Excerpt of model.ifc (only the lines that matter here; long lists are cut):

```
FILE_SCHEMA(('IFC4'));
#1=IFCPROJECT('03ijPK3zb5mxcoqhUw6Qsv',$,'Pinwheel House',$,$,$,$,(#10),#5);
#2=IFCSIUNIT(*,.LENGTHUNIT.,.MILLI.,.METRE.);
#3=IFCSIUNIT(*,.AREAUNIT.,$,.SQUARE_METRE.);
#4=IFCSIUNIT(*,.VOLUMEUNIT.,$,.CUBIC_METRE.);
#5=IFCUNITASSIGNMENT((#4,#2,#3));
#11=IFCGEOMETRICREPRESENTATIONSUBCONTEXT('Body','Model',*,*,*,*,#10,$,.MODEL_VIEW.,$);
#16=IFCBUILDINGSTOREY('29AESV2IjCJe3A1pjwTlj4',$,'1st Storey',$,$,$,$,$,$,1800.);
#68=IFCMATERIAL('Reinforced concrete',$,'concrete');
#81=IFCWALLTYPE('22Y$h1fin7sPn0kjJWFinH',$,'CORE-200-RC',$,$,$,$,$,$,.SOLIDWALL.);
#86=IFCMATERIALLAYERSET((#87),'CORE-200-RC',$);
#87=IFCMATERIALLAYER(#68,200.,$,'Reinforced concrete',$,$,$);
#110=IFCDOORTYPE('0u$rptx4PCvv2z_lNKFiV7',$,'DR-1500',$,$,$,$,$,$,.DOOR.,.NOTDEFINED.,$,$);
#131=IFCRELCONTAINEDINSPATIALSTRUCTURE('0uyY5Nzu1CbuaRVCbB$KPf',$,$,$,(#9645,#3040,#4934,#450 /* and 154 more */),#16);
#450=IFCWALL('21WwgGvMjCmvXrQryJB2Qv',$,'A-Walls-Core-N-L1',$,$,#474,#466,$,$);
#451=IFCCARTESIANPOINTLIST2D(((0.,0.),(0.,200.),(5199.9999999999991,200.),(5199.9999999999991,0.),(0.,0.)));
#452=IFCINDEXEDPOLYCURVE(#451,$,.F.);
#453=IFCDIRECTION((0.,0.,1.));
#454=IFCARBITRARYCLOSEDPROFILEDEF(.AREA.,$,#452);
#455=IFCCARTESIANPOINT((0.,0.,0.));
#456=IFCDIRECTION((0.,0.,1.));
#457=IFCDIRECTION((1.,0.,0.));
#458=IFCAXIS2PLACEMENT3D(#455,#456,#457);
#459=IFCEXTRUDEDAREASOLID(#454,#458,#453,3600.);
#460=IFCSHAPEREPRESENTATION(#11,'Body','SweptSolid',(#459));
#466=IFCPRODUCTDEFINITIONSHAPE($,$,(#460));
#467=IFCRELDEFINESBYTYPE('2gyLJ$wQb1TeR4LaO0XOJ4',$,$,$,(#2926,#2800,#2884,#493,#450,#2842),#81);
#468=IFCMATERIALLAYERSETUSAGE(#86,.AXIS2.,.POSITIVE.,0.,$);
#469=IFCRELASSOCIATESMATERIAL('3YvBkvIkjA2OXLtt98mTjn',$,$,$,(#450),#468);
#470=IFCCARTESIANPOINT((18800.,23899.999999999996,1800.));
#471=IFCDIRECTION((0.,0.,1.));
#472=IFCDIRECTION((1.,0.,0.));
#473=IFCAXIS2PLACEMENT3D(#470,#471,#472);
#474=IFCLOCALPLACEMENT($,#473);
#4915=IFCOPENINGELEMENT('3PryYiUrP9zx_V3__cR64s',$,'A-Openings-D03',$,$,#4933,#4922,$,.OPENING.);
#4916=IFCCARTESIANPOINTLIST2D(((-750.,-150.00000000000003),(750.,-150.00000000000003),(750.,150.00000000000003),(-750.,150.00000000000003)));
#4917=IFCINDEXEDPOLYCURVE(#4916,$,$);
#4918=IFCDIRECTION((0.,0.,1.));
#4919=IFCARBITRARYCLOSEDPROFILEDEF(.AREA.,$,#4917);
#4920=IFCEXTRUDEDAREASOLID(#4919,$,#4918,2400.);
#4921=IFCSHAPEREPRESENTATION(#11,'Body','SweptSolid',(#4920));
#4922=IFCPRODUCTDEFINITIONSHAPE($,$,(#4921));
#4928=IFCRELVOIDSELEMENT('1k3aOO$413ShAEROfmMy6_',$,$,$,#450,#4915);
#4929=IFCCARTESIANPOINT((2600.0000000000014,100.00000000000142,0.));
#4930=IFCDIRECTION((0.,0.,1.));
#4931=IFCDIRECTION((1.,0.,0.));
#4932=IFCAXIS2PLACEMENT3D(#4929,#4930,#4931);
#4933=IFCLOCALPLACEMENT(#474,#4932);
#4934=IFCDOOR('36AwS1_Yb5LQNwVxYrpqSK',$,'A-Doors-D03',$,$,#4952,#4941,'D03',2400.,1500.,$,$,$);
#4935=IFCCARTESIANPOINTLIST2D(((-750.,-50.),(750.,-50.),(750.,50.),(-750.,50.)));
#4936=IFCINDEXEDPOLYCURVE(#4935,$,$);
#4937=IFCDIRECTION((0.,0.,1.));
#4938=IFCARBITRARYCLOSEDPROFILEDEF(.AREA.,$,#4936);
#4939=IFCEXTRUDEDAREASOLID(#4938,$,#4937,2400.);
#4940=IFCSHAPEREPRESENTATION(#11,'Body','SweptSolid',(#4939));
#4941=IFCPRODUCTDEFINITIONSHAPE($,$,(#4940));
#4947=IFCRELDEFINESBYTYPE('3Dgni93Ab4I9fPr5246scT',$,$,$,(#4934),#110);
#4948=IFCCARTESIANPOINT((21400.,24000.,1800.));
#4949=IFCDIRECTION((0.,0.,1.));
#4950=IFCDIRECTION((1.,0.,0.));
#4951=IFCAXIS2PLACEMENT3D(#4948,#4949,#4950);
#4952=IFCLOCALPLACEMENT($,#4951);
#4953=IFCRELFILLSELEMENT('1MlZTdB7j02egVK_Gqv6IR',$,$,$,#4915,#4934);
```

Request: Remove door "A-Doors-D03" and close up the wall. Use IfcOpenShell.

```python
import ifcopenshell
import ifcopenshell.api.feature
import ifcopenshell.api.root
import ifcopenshell.geom
import ifcopenshell.util.shape

model = ifcopenshell.open("model.ifc")
settings = ifcopenshell.geom.settings()


def volume(element):
    """Net volume in cubic metres, openings subtracted."""
    shape = ifcopenshell.geom.create_shape(settings, element)
    return ifcopenshell.util.shape.get_volume(shape.geometry)


door = model.by_guid("36AwS1_Yb5LQNwVxYrpqSK")
opening = door.FillsVoids[0].RelatingOpeningElement
wall = opening.VoidsElements[0].RelatingBuildingElement
before = volume(wall)

ifcopenshell.api.root.remove_product(model, product=door)
ifcopenshell.api.feature.remove_feature(model, feature=opening)

after = volume(wall)

print(f"wall volume {before:.3f} -> {after:.3f} m3")

model.write("model_edited.ifc")
```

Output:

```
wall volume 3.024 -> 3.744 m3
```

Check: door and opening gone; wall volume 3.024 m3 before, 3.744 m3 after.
